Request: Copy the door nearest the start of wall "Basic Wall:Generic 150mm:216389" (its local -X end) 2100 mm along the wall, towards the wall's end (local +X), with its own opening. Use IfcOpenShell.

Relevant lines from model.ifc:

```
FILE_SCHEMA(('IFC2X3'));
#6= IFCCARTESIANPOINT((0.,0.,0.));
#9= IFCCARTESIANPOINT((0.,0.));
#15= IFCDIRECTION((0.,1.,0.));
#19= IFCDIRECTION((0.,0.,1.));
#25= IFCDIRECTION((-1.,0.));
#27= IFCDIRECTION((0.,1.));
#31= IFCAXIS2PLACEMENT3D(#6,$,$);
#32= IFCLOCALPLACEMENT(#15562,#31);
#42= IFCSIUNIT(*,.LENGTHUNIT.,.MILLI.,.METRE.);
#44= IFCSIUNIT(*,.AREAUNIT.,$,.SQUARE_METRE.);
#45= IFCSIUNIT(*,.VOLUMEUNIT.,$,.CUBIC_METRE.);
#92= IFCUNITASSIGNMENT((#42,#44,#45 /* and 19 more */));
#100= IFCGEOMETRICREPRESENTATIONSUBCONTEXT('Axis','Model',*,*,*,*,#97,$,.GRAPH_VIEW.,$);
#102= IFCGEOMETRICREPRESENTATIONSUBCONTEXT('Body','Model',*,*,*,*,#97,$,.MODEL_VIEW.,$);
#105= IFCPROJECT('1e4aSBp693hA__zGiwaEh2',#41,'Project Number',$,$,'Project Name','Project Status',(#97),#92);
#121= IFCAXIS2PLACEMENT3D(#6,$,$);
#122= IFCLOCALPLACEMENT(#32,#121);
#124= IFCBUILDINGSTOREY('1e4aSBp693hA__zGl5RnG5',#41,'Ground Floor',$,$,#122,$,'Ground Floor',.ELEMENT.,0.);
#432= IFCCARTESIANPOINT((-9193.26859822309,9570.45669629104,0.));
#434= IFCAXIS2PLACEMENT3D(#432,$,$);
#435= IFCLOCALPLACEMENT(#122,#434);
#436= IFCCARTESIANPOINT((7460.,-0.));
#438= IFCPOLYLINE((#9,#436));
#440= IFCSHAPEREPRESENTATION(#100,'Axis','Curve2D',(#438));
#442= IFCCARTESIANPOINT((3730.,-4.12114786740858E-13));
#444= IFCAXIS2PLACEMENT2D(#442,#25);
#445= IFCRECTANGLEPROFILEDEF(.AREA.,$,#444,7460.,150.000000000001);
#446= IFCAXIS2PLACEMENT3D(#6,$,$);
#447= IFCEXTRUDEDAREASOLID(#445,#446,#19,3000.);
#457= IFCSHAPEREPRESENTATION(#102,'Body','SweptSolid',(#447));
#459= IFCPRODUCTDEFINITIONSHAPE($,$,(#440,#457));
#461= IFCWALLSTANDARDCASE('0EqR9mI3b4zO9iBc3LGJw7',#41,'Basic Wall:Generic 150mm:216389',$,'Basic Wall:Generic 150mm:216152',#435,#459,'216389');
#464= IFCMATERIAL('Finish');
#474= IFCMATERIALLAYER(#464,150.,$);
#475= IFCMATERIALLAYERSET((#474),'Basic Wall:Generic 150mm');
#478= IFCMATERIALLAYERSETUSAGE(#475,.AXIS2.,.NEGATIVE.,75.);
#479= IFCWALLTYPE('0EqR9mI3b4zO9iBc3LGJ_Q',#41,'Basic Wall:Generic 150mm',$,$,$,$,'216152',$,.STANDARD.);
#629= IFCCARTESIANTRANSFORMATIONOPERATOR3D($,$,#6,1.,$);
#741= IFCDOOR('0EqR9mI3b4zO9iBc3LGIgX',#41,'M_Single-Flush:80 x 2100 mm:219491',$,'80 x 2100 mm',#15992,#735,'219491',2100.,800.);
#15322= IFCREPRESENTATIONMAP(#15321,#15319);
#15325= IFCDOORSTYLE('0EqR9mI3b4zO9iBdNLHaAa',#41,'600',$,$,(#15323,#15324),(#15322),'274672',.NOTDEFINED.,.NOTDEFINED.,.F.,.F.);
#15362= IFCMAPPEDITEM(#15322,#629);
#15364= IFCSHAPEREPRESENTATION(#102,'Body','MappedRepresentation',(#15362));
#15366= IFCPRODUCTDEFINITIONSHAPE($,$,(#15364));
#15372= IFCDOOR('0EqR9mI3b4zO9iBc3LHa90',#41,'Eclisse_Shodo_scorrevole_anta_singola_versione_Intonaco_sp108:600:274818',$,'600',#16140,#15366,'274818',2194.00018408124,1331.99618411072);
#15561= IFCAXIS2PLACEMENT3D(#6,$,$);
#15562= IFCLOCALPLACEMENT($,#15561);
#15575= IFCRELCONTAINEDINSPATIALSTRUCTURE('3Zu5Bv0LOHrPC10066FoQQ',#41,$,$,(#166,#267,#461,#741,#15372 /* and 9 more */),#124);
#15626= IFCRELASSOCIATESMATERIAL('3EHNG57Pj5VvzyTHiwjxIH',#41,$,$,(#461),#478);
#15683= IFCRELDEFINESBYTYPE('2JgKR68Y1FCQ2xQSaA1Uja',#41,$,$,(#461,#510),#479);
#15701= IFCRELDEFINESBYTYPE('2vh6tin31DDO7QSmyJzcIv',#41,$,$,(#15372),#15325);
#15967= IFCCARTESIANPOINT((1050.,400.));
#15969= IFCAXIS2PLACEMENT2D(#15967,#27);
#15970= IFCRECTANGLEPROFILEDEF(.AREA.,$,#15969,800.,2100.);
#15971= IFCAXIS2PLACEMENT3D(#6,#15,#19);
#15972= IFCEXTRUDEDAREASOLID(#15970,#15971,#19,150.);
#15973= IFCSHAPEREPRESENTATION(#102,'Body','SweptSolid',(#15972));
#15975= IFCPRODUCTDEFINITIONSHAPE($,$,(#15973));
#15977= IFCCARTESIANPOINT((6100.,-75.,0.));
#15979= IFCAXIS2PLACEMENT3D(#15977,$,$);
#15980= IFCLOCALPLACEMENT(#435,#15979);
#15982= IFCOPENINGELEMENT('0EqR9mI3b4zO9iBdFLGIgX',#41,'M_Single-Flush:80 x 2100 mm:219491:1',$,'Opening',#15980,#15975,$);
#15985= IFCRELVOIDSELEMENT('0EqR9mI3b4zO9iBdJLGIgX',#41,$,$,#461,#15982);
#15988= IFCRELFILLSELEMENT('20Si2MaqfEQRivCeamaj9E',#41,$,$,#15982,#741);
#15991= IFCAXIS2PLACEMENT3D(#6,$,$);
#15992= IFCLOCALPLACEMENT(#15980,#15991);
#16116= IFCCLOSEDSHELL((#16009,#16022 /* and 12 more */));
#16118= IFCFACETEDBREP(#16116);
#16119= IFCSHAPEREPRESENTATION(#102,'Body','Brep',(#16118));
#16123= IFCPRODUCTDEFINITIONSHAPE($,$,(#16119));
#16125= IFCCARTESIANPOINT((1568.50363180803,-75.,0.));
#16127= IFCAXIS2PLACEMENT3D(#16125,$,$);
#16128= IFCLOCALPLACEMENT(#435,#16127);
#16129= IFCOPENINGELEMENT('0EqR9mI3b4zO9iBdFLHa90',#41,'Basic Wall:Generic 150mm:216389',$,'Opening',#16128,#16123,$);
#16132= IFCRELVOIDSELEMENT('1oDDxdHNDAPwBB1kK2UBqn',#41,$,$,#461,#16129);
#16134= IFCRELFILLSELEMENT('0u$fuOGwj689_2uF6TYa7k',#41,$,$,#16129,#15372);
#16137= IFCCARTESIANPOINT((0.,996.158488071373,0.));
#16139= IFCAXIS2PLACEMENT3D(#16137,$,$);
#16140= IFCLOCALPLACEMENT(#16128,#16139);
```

```python
import ifcopenshell
import ifcopenshell.api.feature
import ifcopenshell.api.geometry
import ifcopenshell.api.root
import ifcopenshell.geom
import ifcopenshell.util.element
import ifcopenshell.util.placement
import ifcopenshell.util.shape
import ifcopenshell.util.unit

model = ifcopenshell.open("model.ifc")
unit_scale = ifcopenshell.util.unit.calculate_unit_scale(model)
settings = ifcopenshell.geom.settings()


def volume(element):
    """Net volume in cubic metres, openings subtracted."""
    shape = ifcopenshell.geom.create_shape(settings, element)
    return ifcopenshell.util.shape.get_volume(shape.geometry)


def reuse_history(source, copy):
    """copy_class also copies each property set's owner history, people and application; keep the originals."""
    for rel in copy.IsDefinedBy:
        if rel.is_a("IfcRelDefinesByProperties") and (history := rel.RelatingPropertyDefinition.OwnerHistory):
            rel.RelatingPropertyDefinition.OwnerHistory = source.OwnerHistory
            ifcopenshell.util.element.remove_deep2(model, history)


door = model.by_id(15372)
opening = door.FillsVoids[0].RelatingOpeningElement
wall = opening.VoidsElements[0].RelatingBuildingElement
before = volume(wall)
shift = ifcopenshell.util.placement.get_local_placement(wall.ObjectPlacement)[:3, 0] * 2.1 / unit_scale

# copy_class copies the void relationship, type, container and properties, but no geometry.
new_opening = ifcopenshell.api.root.copy_class(model, product=opening)
new_opening.Representation = ifcopenshell.util.element.copy_deep(
    model, opening.Representation, exclude=["IfcGeometricRepresentationContext", "IfcRepresentationMap"]
)
new_opening.Name = "Basic Wall:Generic 150mm"
new_door = ifcopenshell.api.root.copy_class(model, product=door)
new_door.Representation = ifcopenshell.util.element.copy_deep(
    model, door.Representation, exclude=["IfcGeometricRepresentationContext", "IfcRepresentationMap"]
)
new_door.Name = "Eclisse_Shodo_scorrevole_anta_singola_versione_Intonaco_sp108:600"
new_door.Tag = None
reuse_history(door, new_door)
fills = ifcopenshell.api.feature.add_filling(model, opening=new_opening, element=new_door)
fills.OwnerHistory = new_door.OwnerHistory  # required in IFC2X3

for old, new in ((opening, new_opening), (door, new_door)):
    matrix = ifcopenshell.util.placement.get_local_placement(old.ObjectPlacement)
    matrix[:3, 3] += shift
    ifcopenshell.api.geometry.edit_object_placement(model, product=new, matrix=matrix, is_si=False)

after = volume(wall)

print(f"wall volume {before:.3f} -> {after:.3f} m3")

model.write("model-out.ifc")
```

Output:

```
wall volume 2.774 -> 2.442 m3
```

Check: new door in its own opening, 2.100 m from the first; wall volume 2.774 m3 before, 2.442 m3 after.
